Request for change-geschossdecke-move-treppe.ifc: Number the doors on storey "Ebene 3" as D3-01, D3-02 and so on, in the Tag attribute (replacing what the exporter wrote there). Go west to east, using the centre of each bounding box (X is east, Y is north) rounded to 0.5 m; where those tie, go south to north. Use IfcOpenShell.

First a look at what the model holds.

```python
import ifcopenshell
import ifcopenshell.util.element
import ifcopenshell.util.placement

model = ifcopenshell.open("change-geschossdecke-move-treppe.ifc")
print(model.schema)
storey = next(s for s in model.by_type("IfcBuildingStorey") if s.Name == "Ebene 3")
doors = [e for e in ifcopenshell.util.element.get_decomposition(storey) if e.is_a("IfcDoor")]
for e in sorted(doors, key=lambda e: e.id()):
    origin = ifcopenshell.util.placement.get_local_placement(e.ObjectPlacement)[:3, 3]
    print(e.id(), e.Tag, e.Name, origin.round(2) + 0.0, sep=" | ")
```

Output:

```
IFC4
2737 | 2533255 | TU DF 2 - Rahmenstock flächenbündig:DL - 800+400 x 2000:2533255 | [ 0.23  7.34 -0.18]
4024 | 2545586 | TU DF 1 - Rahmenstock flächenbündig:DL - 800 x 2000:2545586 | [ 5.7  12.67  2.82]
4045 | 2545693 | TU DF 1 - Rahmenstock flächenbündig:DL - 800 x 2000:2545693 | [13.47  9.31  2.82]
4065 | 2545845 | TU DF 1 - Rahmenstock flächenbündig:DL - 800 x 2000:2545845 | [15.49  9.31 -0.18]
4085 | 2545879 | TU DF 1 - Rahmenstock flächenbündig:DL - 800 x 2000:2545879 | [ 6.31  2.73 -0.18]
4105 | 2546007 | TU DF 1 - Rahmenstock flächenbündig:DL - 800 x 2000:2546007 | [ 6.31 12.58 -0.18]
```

```python
import ifcopenshell
import ifcopenshell.geom
import ifcopenshell.util.element
import ifcopenshell.util.shape

model = ifcopenshell.open("change-geschossdecke-move-treppe.ifc")
settings = ifcopenshell.geom.settings()
settings.set("use-world-coords", True)


def centre(element):
    shape = ifcopenshell.geom.create_shape(settings, element)
    return ifcopenshell.util.shape.get_bbox_centroid(shape.geometry)


storey = next(s for s in model.by_type("IfcBuildingStorey") if s.Name == "Ebene 3")
doors = [e for e in ifcopenshell.util.element.get_decomposition(storey) if e.is_a("IfcDoor")]

# Insertion points can sit at a corner or the storey origin, so sort by the geometry (in metres).
centres = {e: centre(e) for e in doors}
doors.sort(key=lambda e: (round(centres[e][0] / 0.5), centres[e][1]))

for i, e in enumerate(doors, start=1):
    number = f"D3-{i:02d}"
    e.Tag = number
    print(e.id(), number)

model.write("change-geschossdecke-move-treppe-out.ifc")
```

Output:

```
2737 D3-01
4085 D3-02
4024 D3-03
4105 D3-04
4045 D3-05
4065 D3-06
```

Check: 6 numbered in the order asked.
